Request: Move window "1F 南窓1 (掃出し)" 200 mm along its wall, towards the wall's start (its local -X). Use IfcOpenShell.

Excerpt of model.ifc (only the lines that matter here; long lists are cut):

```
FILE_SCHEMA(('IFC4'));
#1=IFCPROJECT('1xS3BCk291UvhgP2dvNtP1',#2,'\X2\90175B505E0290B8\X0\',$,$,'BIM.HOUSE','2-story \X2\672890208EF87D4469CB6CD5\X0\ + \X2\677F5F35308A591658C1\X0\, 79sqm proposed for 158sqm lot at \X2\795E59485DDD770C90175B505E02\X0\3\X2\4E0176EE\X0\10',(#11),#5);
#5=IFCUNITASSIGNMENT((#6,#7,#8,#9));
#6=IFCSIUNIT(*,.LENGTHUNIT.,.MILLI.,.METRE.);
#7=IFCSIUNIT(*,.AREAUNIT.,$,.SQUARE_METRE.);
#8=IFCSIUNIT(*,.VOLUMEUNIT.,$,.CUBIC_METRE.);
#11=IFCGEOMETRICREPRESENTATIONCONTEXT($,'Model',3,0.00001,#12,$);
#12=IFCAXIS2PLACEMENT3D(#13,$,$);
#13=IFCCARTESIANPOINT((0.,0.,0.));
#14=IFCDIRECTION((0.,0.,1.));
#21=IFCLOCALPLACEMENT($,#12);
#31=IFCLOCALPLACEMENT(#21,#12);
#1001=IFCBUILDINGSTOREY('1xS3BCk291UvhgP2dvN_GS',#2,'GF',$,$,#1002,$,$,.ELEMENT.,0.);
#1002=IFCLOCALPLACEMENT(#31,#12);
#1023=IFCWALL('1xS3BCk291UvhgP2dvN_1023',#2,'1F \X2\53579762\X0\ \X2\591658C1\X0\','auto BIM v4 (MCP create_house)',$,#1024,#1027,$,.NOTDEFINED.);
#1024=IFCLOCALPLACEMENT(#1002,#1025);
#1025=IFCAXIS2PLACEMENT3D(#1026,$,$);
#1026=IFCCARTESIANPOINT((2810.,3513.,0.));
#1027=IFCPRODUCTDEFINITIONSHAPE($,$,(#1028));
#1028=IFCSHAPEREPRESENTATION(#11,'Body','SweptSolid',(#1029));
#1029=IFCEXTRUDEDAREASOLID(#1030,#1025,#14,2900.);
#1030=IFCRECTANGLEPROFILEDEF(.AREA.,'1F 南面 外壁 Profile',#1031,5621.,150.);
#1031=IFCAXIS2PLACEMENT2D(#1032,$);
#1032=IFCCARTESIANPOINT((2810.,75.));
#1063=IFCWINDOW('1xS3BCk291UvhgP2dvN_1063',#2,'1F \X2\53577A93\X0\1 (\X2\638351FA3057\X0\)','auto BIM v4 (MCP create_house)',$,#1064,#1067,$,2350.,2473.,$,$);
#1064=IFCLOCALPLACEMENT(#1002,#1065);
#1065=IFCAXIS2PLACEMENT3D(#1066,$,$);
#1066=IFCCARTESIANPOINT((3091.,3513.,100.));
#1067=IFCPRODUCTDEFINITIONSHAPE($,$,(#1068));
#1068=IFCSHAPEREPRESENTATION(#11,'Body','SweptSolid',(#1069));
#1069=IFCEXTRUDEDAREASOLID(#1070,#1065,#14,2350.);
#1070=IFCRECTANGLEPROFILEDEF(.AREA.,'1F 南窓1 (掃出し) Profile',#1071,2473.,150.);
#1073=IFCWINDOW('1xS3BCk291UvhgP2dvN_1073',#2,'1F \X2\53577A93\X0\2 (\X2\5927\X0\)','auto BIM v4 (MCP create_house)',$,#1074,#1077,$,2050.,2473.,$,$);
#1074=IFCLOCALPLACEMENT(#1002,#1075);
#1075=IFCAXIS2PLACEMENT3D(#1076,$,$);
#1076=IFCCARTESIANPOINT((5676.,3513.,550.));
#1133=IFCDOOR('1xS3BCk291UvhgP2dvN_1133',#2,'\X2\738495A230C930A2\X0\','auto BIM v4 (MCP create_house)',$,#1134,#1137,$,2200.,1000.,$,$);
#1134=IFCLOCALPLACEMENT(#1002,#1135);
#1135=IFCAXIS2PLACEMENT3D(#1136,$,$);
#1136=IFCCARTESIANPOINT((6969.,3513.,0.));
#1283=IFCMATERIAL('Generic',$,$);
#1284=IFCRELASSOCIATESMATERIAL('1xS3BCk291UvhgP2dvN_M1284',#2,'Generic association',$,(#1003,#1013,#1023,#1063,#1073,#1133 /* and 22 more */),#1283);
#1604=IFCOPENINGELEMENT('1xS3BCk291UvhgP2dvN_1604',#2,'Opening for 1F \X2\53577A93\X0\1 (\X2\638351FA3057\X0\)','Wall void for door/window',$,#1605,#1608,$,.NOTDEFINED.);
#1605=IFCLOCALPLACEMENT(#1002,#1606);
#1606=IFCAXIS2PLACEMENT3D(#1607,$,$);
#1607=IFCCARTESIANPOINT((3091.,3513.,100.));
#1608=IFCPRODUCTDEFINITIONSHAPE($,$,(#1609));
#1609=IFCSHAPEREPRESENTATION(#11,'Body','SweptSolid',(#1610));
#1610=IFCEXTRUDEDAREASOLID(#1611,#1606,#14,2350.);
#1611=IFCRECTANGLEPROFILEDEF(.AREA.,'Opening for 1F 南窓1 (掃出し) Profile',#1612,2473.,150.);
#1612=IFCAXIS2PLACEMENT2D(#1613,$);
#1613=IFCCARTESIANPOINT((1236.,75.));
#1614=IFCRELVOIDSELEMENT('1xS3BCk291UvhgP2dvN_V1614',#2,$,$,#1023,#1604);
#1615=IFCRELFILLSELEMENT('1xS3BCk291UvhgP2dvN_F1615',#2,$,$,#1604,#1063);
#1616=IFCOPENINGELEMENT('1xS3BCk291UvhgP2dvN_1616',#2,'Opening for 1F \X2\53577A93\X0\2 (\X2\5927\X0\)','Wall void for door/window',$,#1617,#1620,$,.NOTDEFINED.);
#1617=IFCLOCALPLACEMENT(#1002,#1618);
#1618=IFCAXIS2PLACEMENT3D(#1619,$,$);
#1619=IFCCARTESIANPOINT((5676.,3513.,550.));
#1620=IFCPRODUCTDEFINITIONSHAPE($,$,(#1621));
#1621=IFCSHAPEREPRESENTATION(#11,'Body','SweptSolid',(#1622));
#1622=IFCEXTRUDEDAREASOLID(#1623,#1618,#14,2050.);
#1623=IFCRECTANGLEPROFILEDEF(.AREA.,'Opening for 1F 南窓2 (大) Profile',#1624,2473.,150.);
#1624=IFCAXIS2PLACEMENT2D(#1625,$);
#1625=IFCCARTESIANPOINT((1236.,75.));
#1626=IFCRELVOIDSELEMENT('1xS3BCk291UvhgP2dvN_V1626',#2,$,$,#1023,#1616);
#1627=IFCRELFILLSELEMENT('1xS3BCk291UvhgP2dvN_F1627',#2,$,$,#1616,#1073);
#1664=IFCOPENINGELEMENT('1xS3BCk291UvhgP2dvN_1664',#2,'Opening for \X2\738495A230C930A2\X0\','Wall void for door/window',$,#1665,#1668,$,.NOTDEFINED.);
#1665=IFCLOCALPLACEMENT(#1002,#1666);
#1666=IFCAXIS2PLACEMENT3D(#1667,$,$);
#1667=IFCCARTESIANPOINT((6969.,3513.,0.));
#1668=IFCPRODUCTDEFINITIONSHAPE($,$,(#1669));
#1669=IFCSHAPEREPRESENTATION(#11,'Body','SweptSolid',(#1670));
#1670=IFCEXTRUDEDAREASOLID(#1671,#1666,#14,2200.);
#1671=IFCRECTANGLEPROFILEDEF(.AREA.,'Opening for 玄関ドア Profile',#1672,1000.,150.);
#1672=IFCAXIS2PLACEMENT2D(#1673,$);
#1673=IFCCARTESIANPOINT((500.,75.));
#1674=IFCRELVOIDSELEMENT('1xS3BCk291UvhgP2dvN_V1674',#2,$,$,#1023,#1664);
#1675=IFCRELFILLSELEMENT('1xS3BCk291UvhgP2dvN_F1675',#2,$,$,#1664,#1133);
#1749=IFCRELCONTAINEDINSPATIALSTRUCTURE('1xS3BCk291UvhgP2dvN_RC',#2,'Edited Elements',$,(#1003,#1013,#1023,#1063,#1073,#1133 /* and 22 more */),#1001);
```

```python
import ifcopenshell
import ifcopenshell.api.geometry
import ifcopenshell.util.placement

model = ifcopenshell.open("model.ifc")

window = model.by_id(1063)
opening = window.FillsVoids[0].RelatingOpeningElement
wall = opening.VoidsElements[0].RelatingBuildingElement

wall_matrix = ifcopenshell.util.placement.get_local_placement(wall.ObjectPlacement)
shift = wall_matrix[:3, 0] * -200.0
before = ifcopenshell.util.placement.get_local_placement(window.ObjectPlacement)[:3, 3].copy()

# The window is not placed relative to its opening, so move both.
for product in (opening, window):
    matrix = ifcopenshell.util.placement.get_local_placement(product.ObjectPlacement)
    matrix[:3, 3] += shift
    ifcopenshell.api.geometry.edit_object_placement(model, product=product, matrix=matrix, is_si=False)

after = ifcopenshell.util.placement.get_local_placement(window.ObjectPlacement)[:3, 3]
print("window moved by", (after - before).round(3) + 0.0)

model.write("model_updated.ifc")
```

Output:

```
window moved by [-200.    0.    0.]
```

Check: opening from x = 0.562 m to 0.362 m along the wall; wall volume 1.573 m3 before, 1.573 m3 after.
